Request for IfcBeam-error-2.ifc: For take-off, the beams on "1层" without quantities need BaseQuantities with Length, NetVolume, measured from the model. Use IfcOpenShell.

First a look at what the model holds.

```python
import ifcopenshell
import ifcopenshell.util.element
import ifcopenshell.util.unit

model = ifcopenshell.open("IfcBeam-error-2.ifc")
print(model.schema)
for unit_type in ("LENGTHUNIT", "AREAUNIT", "VOLUMEUNIT"):
    print(unit_type, ifcopenshell.util.unit.calculate_unit_scale(model, unit_type))
storey = next(s for s in model.by_type("IfcBuildingStorey") if s.Name == "1层")
beams = [e for e in ifcopenshell.util.element.get_decomposition(storey) if e.is_a("IfcBeam")]
for e in sorted(beams, key=lambda e: e.id()):
    print(e.id(), e.is_a(), e.Name, list(ifcopenshell.util.element.get_psets(e, qtos_only=True)), sep=" | ")
```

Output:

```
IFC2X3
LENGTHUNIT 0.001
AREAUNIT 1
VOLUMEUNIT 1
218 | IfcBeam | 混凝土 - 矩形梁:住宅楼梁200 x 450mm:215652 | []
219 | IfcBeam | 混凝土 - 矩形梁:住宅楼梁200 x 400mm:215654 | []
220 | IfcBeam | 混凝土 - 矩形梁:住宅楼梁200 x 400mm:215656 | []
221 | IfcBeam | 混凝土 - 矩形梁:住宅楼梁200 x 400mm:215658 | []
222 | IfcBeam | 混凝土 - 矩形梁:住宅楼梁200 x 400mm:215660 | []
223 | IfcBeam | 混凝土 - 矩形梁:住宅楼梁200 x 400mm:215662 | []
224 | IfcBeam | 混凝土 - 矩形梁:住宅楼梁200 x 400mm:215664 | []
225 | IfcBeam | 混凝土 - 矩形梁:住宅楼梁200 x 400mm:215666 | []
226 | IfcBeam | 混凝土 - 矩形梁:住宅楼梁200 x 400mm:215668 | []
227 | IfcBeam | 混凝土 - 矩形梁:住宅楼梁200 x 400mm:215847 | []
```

```python
import ifcopenshell
import ifcopenshell.api.pset
import ifcopenshell.geom
import ifcopenshell.util.element
import ifcopenshell.util.shape
import ifcopenshell.util.unit

model = ifcopenshell.open("IfcBeam-error-2.ifc")
unit_scale = ifcopenshell.util.unit.calculate_unit_scale(model)
volume_scale = ifcopenshell.util.unit.calculate_unit_scale(model, "VOLUMEUNIT")
settings = ifcopenshell.geom.settings()

storey = next(s for s in model.by_type("IfcBuildingStorey") if s.Name == "1层")
beams = [e for e in ifcopenshell.util.element.get_decomposition(storey) if e.is_a("IfcBeam")]

for e in sorted(beams, key=lambda e: e.id()):
    if ifcopenshell.util.element.get_psets(e, qtos_only=True, should_inherit=False):
        continue
    # Geometry comes back in metres, in the element's own axes.
    shape = ifcopenshell.geom.create_shape(settings, e)
    values = {
        "Length": ifcopenshell.util.shape.get_max_xyz(shape.geometry) / unit_scale,
        "NetVolume": ifcopenshell.util.shape.get_volume(shape.geometry) / volume_scale,
    }
    qto = ifcopenshell.api.pset.add_qto(model, product=e, name="BaseQuantities")
    ifcopenshell.api.pset.edit_qto(model, qto=qto, properties=values)
    print(e.id(), {k: round(v, 3) for k, v in values.items()})

model.write("IfcBeam-error-2_rev.ifc")
```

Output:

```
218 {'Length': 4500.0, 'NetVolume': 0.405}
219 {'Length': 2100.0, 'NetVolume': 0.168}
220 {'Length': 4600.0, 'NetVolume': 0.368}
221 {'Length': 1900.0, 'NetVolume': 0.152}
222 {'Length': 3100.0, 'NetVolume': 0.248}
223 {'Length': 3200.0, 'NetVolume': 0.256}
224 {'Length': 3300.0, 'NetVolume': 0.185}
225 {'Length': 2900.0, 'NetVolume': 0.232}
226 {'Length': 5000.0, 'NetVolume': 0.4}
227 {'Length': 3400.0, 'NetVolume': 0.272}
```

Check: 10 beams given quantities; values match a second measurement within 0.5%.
